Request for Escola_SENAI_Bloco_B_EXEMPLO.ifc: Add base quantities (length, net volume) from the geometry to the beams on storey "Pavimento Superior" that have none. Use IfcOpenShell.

First a look at what the model holds.

```python
import ifcopenshell
import ifcopenshell.util.element
import ifcopenshell.util.unit

model = ifcopenshell.open("Escola_SENAI_Bloco_B_EXEMPLO.ifc")
print(model.schema)
for unit_type in ("LENGTHUNIT", "AREAUNIT", "VOLUMEUNIT"):
    print(unit_type, ifcopenshell.util.unit.calculate_unit_scale(model, unit_type))
storey = next(s for s in model.by_type("IfcBuildingStorey") if s.Name == "Pavimento Superior")
beams = [e for e in ifcopenshell.util.element.get_decomposition(storey) if e.is_a("IfcBeam")]
for e in sorted(beams, key=lambda e: e.id()):
    print(e.id(), e.is_a(), e.Name, list(ifcopenshell.util.element.get_psets(e, qtos_only=True)), sep=" | ")
```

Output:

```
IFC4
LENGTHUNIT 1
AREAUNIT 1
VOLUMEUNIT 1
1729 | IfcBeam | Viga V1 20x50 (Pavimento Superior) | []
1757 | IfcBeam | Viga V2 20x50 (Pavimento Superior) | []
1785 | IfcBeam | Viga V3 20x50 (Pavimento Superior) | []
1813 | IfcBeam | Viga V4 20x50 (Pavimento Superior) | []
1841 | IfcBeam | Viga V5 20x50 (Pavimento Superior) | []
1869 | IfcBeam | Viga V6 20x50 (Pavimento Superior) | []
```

```python
import ifcopenshell
import ifcopenshell.api.pset
import ifcopenshell.geom
import ifcopenshell.util.element
import ifcopenshell.util.shape
import ifcopenshell.util.unit

model = ifcopenshell.open("Escola_SENAI_Bloco_B_EXEMPLO.ifc")
unit_scale = ifcopenshell.util.unit.calculate_unit_scale(model)
volume_scale = ifcopenshell.util.unit.calculate_unit_scale(model, "VOLUMEUNIT")
settings = ifcopenshell.geom.settings()

storey = next(s for s in model.by_type("IfcBuildingStorey") if s.Name == "Pavimento Superior")
beams = [e for e in ifcopenshell.util.element.get_decomposition(storey) if e.is_a("IfcBeam")]

for e in sorted(beams, key=lambda e: e.id()):
    if ifcopenshell.util.element.get_psets(e, qtos_only=True, should_inherit=False):
        continue
    # Geometry comes back in metres, in the element's own axes.
    shape = ifcopenshell.geom.create_shape(settings, e)
    values = {
        "Length": ifcopenshell.util.shape.get_max_xyz(shape.geometry) / unit_scale,
        "NetVolume": ifcopenshell.util.shape.get_volume(shape.geometry) / volume_scale,
    }
    qto = ifcopenshell.api.pset.add_qto(model, product=e, name="Qto_BeamBaseQuantities")
    ifcopenshell.api.pset.edit_qto(model, qto=qto, properties=values)
    print(e.id(), {k: round(v, 3) for k, v in values.items()})

model.write("Escola_SENAI_Bloco_B_EXEMPLO_rev.ifc")
```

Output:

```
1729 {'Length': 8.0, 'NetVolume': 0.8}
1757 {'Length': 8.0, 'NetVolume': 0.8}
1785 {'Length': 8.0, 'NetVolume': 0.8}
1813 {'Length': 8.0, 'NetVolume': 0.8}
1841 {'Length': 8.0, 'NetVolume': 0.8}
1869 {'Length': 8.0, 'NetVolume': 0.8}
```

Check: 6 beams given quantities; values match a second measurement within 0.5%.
